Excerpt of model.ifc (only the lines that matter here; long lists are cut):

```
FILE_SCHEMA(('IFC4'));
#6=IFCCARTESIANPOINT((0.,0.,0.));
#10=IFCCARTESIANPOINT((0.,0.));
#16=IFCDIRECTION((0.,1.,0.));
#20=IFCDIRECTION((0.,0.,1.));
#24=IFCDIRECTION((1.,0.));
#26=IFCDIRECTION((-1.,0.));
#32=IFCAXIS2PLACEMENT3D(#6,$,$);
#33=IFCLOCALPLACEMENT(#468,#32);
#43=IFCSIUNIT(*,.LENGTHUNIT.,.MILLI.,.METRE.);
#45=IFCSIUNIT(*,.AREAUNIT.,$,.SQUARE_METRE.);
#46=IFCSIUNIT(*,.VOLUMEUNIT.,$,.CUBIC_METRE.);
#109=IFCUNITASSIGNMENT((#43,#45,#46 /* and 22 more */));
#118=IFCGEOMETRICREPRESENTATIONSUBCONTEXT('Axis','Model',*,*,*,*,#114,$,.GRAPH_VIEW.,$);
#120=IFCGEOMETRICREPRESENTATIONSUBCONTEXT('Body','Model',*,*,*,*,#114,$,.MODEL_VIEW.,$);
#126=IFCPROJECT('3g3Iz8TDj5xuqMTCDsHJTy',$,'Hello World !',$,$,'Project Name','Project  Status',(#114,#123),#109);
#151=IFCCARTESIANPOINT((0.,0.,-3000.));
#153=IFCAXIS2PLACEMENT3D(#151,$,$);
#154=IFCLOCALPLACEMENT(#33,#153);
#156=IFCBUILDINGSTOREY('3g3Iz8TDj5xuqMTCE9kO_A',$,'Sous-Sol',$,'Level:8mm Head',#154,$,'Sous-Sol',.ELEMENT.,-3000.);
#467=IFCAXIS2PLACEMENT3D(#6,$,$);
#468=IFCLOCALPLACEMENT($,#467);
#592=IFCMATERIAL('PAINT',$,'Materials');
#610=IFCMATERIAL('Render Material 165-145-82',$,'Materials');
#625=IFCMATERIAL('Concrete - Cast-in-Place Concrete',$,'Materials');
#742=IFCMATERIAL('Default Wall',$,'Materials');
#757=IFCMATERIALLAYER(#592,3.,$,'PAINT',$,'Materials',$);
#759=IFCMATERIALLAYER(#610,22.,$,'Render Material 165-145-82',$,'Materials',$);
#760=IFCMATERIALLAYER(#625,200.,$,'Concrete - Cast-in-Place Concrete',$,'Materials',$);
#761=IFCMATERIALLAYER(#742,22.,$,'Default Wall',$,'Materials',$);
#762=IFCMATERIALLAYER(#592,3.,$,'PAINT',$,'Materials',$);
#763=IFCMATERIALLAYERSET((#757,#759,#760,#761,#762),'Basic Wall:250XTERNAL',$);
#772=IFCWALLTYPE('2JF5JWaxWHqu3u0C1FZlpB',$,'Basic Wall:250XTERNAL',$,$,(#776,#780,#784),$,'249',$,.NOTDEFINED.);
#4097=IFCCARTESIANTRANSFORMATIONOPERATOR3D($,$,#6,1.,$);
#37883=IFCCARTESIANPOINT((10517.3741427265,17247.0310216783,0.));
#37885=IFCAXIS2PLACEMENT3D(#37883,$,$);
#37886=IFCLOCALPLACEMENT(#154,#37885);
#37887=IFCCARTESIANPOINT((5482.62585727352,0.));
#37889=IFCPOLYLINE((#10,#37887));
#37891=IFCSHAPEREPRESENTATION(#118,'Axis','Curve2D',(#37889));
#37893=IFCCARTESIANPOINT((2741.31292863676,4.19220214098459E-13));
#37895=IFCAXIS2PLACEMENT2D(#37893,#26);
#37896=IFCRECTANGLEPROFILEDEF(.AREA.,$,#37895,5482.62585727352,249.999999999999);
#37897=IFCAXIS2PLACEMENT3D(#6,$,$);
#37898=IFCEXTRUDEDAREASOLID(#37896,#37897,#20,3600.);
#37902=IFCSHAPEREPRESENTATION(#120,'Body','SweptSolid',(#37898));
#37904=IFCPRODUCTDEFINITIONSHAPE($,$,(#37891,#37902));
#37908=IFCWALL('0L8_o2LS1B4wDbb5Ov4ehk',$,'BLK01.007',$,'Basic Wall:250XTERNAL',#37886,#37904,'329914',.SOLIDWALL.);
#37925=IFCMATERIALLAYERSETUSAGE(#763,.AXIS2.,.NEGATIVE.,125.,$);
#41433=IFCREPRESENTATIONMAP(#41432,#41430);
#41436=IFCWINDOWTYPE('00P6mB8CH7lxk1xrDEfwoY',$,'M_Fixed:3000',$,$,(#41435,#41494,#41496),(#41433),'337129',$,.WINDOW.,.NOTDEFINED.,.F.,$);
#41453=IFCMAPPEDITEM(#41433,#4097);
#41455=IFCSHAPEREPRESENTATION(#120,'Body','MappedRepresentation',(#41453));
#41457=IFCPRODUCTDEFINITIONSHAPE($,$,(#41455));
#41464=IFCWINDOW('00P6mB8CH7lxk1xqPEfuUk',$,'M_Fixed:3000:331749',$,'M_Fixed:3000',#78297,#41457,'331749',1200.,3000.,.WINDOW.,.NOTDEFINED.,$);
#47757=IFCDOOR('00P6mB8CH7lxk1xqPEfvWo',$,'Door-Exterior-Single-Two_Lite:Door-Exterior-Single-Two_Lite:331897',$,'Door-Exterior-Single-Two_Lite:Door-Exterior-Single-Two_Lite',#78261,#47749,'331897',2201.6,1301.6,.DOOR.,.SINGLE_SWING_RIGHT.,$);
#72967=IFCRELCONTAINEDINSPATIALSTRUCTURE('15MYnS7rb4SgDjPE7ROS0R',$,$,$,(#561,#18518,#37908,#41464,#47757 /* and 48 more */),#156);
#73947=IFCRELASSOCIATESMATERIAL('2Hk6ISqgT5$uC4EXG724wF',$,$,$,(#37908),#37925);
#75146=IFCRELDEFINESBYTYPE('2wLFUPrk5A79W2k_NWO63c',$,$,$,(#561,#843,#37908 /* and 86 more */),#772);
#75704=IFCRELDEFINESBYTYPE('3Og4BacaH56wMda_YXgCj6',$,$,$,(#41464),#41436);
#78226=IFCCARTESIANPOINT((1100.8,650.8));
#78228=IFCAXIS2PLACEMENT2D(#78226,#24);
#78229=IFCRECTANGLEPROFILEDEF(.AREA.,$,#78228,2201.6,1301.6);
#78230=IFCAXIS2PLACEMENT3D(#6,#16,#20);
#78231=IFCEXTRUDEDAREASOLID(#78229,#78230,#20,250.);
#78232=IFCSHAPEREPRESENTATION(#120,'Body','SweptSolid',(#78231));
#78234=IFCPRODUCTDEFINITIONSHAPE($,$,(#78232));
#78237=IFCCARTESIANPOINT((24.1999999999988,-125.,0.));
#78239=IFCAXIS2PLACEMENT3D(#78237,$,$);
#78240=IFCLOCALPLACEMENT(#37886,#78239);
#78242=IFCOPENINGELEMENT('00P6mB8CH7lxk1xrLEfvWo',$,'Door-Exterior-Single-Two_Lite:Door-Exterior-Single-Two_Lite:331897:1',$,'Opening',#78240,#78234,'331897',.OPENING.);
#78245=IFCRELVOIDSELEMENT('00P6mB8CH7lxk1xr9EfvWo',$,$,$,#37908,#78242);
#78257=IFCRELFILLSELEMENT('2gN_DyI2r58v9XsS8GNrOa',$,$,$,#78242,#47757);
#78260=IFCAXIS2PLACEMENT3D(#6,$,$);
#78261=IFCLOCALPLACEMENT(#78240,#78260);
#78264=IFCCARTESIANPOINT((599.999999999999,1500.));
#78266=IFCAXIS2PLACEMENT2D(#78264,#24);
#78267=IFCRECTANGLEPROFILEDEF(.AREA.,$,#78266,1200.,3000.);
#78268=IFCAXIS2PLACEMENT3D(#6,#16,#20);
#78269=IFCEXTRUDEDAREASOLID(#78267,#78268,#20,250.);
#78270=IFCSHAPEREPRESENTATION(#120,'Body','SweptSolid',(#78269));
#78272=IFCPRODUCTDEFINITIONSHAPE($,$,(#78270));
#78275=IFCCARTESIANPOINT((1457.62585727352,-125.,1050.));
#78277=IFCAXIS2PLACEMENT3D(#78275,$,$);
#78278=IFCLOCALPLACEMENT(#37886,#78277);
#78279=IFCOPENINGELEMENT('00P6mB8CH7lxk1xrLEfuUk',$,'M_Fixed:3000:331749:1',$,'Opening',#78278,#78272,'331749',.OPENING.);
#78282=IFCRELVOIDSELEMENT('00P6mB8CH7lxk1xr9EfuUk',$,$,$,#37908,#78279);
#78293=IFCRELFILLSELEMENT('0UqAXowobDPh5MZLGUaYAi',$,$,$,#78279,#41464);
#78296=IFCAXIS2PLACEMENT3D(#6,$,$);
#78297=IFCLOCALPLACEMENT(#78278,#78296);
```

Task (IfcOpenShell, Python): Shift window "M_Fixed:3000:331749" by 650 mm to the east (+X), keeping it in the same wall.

```python
import ifcopenshell
import ifcopenshell.api.geometry
import ifcopenshell.util.placement
import ifcopenshell.util.unit

model = ifcopenshell.open("model.ifc")
unit_scale = ifcopenshell.util.unit.calculate_unit_scale(model)

window = model.by_id(41464)
opening = window.FillsVoids[0].RelatingOpeningElement
wall = opening.VoidsElements[0].RelatingBuildingElement

wall_matrix = ifcopenshell.util.placement.get_local_placement(wall.ObjectPlacement)
shift = wall_matrix[:3, 0] * 0.65 / unit_scale
before = ifcopenshell.util.placement.get_local_placement(window.ObjectPlacement)[:3, 3].copy()

# The window is placed relative to its opening, so it follows when the opening moves.
matrix = ifcopenshell.util.placement.get_local_placement(opening.ObjectPlacement)
matrix[:3, 3] += shift
ifcopenshell.api.geometry.edit_object_placement(
    model, product=opening, matrix=matrix, is_si=False, should_transform_children=True
)

after = ifcopenshell.util.placement.get_local_placement(window.ObjectPlacement)[:3, 3]
print("window moved by", (after - before).round(3) + 0.0)

model.write("model_updated.ifc")
```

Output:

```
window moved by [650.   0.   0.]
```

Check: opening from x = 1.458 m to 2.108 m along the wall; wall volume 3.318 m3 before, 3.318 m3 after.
